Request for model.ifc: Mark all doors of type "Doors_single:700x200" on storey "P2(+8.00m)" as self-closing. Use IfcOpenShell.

First a look at what the model holds.

```python
import ifcopenshell
import ifcopenshell.util.element

model = ifcopenshell.open("model.ifc")
print(model.schema)
storey = next(s for s in model.by_type("IfcBuildingStorey") if s.Name == "P2(+8.00m)")
doors = [e for e in ifcopenshell.util.element.get_decomposition(storey) if e.is_a("IfcDoor")]
seen = {}
for e in doors:
    element_type = ifcopenshell.util.element.get_type(e)
    key = (element_type.Name if element_type != e and element_type else None, ifcopenshell.util.element.get_pset(e, "Pset_DoorCommon", "SelfClosing"))
    seen[key] = seen.get(key, 0) + 1
for (name, value), count in sorted(seen.items(), key=str):
    print(count, "x", name, "|", value)
```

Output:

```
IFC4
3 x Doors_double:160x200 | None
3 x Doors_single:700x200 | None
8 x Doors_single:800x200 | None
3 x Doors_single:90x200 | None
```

```python
import ifcopenshell
import ifcopenshell.api.pset
import ifcopenshell.util.element

model = ifcopenshell.open("model.ifc")

storey = next(s for s in model.by_type("IfcBuildingStorey") if s.Name == "P2(+8.00m)")
doors = [e for e in ifcopenshell.util.element.get_decomposition(storey) if e.is_a("IfcDoor")]

count = 0
for e in doors:
    element_type = ifcopenshell.util.element.get_type(e)
    if element_type in (None, e) or element_type.Name != "Doors_single:700x200":
        continue
    # add_pset returns the element's existing set when there is one.
    pset = ifcopenshell.api.pset.add_pset(model, product=e, name="Pset_DoorCommon")
    ifcopenshell.api.pset.edit_pset(model, pset=pset, properties={"SelfClosing": True})
    count += 1

print(count, "doors updated")

model.write("model_v2.ifc")
```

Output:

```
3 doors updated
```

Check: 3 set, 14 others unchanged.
